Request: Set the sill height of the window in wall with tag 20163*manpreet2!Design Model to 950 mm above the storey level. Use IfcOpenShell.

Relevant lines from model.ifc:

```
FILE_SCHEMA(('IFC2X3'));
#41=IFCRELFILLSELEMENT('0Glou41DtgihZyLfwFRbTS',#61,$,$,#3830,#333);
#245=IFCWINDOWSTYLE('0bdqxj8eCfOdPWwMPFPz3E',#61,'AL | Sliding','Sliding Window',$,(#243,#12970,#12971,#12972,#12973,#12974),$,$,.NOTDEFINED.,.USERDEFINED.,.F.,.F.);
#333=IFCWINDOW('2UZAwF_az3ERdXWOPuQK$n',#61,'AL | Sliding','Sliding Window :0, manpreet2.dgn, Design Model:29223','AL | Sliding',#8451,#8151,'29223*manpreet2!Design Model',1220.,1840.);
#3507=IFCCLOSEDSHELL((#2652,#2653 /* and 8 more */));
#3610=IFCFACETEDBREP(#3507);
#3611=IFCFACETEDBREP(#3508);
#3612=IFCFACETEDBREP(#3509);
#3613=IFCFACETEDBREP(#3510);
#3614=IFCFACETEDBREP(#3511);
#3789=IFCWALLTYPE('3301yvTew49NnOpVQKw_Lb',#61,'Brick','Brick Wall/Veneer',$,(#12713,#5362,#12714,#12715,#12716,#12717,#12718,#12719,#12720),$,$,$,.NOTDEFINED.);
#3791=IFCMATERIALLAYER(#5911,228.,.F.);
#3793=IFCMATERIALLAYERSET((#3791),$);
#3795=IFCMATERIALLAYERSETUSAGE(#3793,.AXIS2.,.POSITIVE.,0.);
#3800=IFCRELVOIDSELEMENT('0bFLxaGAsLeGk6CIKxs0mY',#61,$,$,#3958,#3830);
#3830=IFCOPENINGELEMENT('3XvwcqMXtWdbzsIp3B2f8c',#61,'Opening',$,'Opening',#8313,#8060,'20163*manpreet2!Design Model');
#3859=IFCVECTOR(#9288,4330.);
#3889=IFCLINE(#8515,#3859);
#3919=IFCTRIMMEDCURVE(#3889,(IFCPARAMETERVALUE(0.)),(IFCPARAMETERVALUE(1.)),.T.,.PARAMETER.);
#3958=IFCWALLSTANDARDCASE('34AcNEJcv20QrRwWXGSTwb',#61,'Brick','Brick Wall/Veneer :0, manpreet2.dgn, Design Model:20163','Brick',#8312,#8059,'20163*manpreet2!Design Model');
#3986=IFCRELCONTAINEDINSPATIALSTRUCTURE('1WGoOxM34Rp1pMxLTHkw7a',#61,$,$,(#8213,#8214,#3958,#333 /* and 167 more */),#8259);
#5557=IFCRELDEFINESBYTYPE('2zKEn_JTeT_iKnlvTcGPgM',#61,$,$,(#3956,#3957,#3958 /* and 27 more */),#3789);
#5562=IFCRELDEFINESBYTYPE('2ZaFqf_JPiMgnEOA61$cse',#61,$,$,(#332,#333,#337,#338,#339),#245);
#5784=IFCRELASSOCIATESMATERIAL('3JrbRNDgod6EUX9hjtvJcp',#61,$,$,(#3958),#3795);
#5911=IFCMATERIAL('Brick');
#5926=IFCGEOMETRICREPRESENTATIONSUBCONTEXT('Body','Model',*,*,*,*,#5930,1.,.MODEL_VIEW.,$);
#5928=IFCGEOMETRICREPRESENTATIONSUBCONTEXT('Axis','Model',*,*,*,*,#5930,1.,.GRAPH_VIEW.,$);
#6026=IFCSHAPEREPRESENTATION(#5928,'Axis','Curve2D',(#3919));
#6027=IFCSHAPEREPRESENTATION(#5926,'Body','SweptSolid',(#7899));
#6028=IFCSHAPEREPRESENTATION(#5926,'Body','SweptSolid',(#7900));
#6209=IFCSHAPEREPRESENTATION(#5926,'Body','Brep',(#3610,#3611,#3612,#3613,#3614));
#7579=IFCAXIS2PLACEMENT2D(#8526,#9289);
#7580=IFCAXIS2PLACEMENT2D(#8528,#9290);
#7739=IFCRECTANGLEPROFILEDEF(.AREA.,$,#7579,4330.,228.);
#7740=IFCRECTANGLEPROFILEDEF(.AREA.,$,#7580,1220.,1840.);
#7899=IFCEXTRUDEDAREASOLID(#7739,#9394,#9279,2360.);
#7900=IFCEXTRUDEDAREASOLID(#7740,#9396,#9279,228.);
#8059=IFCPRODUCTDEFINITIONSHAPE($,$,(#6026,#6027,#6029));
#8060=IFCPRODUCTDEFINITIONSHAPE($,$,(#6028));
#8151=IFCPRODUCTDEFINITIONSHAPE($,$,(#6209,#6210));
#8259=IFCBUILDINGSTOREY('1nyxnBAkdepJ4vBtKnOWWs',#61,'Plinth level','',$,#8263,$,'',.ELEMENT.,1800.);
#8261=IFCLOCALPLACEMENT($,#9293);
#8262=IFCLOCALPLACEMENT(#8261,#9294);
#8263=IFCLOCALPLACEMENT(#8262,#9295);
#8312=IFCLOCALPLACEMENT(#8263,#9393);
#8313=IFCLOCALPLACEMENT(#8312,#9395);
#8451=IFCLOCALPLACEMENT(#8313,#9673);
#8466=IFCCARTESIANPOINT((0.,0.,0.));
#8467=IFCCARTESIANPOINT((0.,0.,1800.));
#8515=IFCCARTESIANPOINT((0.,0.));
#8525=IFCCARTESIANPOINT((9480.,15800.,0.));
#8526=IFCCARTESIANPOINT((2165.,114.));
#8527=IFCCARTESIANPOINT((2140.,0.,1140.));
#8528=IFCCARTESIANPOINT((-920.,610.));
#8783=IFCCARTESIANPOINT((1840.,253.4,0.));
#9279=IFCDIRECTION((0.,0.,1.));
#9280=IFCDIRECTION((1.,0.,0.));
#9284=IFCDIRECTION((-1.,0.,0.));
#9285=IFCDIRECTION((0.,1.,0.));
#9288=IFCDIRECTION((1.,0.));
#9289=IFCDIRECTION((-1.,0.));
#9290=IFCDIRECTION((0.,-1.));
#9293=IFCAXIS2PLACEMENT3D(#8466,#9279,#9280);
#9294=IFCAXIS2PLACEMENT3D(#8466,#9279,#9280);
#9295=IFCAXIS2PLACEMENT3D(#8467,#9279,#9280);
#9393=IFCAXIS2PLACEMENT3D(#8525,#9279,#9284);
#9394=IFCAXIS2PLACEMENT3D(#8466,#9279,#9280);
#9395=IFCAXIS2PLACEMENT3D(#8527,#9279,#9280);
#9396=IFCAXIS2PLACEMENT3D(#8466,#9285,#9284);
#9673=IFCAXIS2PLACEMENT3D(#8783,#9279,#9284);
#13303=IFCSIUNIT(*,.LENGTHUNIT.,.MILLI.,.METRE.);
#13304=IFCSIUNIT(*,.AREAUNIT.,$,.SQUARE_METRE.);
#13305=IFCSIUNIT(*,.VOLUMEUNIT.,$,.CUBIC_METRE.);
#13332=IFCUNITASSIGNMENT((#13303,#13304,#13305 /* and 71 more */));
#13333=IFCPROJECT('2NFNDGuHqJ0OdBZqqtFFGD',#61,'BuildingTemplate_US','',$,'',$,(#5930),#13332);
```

```python
import numpy as np
import ifcopenshell
import ifcopenshell.api.geometry
import ifcopenshell.geom
import ifcopenshell.util.element
import ifcopenshell.util.placement
import ifcopenshell.util.shape
import ifcopenshell.util.unit

model = ifcopenshell.open("model.ifc")
unit_scale = ifcopenshell.util.unit.calculate_unit_scale(model)

window = model.by_guid("2UZAwF_az3ERdXWOPuQK$n")
opening = window.FillsVoids[0].RelatingOpeningElement
storey = ifcopenshell.util.element.get_container(window, ifc_class="IfcBuildingStorey")
level = ifcopenshell.util.placement.get_local_placement(storey.ObjectPlacement)[2, 3]

# The opening's origin need not be at the sill, so measure its lowest point.
shape = ifcopenshell.geom.create_shape(ifcopenshell.geom.settings(), opening)
bottom = ifcopenshell.util.shape.get_shape_bottom_elevation(shape, shape.geometry) / unit_scale
dz = level + 0.95 / unit_scale - bottom

shift = np.array([0.0, 0.0, dz])
# The window is placed relative to its opening, so it follows when the opening moves.
matrix = ifcopenshell.util.placement.get_local_placement(opening.ObjectPlacement)
matrix[:3, 3] += shift
ifcopenshell.api.geometry.edit_object_placement(
    model, product=opening, matrix=matrix, is_si=False, should_transform_children=True
)

print(f"moved by {dz * unit_scale:+.3f} m")

model.write("model-out.ifc")
```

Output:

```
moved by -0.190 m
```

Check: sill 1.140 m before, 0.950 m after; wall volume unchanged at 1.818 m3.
